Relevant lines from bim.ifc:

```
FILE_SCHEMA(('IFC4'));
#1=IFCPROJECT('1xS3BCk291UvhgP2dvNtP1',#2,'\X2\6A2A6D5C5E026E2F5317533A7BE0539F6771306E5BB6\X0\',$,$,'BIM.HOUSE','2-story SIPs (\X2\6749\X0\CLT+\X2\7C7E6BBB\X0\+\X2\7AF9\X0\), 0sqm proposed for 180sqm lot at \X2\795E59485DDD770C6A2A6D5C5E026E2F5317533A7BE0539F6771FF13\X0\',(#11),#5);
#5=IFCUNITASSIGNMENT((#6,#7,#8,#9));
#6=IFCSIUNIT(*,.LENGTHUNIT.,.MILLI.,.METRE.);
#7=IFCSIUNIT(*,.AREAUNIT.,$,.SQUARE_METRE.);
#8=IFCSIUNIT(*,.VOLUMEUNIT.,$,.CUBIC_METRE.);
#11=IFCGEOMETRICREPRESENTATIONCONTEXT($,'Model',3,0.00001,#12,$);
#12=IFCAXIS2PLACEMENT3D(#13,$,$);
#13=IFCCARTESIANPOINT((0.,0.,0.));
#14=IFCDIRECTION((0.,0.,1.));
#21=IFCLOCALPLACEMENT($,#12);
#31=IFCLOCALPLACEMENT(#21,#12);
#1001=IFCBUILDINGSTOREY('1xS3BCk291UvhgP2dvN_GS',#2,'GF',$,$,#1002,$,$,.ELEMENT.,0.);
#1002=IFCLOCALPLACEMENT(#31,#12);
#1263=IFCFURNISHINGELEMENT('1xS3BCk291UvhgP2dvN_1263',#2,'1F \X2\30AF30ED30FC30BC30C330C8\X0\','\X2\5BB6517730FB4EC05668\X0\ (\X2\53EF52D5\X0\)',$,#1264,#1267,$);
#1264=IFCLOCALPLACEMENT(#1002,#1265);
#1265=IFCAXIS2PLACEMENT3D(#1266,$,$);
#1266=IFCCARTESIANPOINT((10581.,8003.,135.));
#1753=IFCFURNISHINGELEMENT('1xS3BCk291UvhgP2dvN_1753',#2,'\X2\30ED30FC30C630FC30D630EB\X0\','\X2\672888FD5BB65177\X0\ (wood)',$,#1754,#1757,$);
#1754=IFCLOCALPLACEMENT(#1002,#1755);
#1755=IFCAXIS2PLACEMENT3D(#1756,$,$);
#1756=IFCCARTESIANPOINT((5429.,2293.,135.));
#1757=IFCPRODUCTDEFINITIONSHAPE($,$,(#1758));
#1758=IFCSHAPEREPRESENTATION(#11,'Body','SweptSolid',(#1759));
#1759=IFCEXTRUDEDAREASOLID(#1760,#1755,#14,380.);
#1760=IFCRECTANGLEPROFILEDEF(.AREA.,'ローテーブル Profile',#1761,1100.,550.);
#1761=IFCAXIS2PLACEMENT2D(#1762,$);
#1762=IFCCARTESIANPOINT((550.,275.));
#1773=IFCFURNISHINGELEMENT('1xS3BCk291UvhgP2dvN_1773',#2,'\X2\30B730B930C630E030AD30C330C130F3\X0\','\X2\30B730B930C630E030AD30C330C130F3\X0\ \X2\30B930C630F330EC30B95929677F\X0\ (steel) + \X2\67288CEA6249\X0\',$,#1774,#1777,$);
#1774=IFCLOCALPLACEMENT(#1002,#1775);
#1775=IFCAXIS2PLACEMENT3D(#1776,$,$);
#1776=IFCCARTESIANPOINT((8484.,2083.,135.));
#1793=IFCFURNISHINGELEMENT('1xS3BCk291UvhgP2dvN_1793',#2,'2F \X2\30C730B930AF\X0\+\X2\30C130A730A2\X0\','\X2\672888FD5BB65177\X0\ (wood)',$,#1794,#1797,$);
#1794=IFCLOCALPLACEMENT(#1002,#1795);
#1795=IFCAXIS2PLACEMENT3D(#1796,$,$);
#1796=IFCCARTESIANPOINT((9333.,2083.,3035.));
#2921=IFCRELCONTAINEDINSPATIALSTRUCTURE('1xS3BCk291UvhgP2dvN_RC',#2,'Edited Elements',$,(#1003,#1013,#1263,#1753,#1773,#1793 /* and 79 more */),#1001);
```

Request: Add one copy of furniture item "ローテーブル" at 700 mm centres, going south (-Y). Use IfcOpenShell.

```python
import numpy as np
import ifcopenshell
import ifcopenshell.api.geometry
import ifcopenshell.api.root
import ifcopenshell.util.element
import ifcopenshell.util.placement

model = ifcopenshell.open("bim.ifc")


def reuse_history(source, copy):
    """copy_class also copies each property set's owner history, people and application; keep the originals."""
    for rel in copy.IsDefinedBy:
        if rel.is_a("IfcRelDefinesByProperties") and (history := rel.RelatingPropertyDefinition.OwnerHistory):
            rel.RelatingPropertyDefinition.OwnerHistory = source.OwnerHistory
            ifcopenshell.util.element.remove_deep2(model, history)


source = model.by_guid("1xS3BCk291UvhgP2dvN_1753")
base = ifcopenshell.util.placement.get_local_placement(source.ObjectPlacement)
step = np.array([0.0, -1.0, 0.0]) * 700.0

for i in range(1, 2):
    copy = ifcopenshell.api.root.copy_class(model, product=source)
    copy.Representation = ifcopenshell.util.element.copy_deep(
        model, source.Representation, exclude=["IfcGeometricRepresentationContext", "IfcRepresentationMap"]
    )
    reuse_history(source, copy)
    matrix = base.copy()
    matrix[:3, 3] += i * step
    print("added at", matrix[:3, 3].round(3) + 0.0)
    ifcopenshell.api.geometry.edit_object_placement(model, product=copy, matrix=matrix, is_si=False)

model.write("bim-out.ifc")
```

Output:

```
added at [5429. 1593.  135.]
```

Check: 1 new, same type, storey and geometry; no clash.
